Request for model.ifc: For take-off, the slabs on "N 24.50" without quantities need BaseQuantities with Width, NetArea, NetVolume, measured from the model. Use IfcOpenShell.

First a look at what the model holds.

```python
import ifcopenshell
import ifcopenshell.util.element
import ifcopenshell.util.unit

model = ifcopenshell.open("model.ifc")
print(model.schema)
for unit_type in ("LENGTHUNIT", "AREAUNIT", "VOLUMEUNIT"):
    print(unit_type, ifcopenshell.util.unit.calculate_unit_scale(model, unit_type))
storey = next(s for s in model.by_type("IfcBuildingStorey") if s.Name == "N 24.50")
slabs = [e for e in ifcopenshell.util.element.get_decomposition(storey) if e.is_a("IfcSlab")]
for e in sorted(slabs, key=lambda e: e.id()):
    print(e.id(), e.is_a(), e.Name, list(ifcopenshell.util.element.get_psets(e, qtos_only=True)), sep=" | ")
```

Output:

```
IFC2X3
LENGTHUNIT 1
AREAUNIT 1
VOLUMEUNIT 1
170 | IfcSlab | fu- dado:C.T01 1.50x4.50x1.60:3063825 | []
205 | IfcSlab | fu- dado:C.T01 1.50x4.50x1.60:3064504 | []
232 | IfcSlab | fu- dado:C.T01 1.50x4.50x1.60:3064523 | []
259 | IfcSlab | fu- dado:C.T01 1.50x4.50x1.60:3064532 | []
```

```python
import ifcopenshell
import ifcopenshell.api.pset
import ifcopenshell.geom
import ifcopenshell.util.element
import ifcopenshell.util.shape
import ifcopenshell.util.unit

model = ifcopenshell.open("model.ifc")
unit_scale = ifcopenshell.util.unit.calculate_unit_scale(model)
area_scale = ifcopenshell.util.unit.calculate_unit_scale(model, "AREAUNIT")
volume_scale = ifcopenshell.util.unit.calculate_unit_scale(model, "VOLUMEUNIT")
settings = ifcopenshell.geom.settings()

storey = next(s for s in model.by_type("IfcBuildingStorey") if s.Name == "N 24.50")
slabs = [e for e in ifcopenshell.util.element.get_decomposition(storey) if e.is_a("IfcSlab")]

for e in sorted(slabs, key=lambda e: e.id()):
    if ifcopenshell.util.element.get_psets(e, qtos_only=True, should_inherit=False):
        continue
    # Geometry comes back in metres, in the element's own axes.
    shape = ifcopenshell.geom.create_shape(settings, e)
    values = {
        "Width": ifcopenshell.util.shape.get_z(shape.geometry) / unit_scale,
        "NetArea": ifcopenshell.util.shape.get_footprint_area(shape.geometry) / area_scale,
        "NetVolume": ifcopenshell.util.shape.get_volume(shape.geometry) / volume_scale,
    }
    qto = ifcopenshell.api.pset.add_qto(model, product=e, name="BaseQuantities")
    ifcopenshell.api.pset.edit_qto(model, qto=qto, properties=values)
    print(e.id(), {k: round(v, 3) for k, v in values.items()})

model.write("model_edited.ifc")
```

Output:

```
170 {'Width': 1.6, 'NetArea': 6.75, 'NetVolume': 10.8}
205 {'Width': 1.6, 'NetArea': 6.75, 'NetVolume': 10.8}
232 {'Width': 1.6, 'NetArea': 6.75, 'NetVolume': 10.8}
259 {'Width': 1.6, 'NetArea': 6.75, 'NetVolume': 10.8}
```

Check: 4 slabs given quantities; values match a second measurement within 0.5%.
